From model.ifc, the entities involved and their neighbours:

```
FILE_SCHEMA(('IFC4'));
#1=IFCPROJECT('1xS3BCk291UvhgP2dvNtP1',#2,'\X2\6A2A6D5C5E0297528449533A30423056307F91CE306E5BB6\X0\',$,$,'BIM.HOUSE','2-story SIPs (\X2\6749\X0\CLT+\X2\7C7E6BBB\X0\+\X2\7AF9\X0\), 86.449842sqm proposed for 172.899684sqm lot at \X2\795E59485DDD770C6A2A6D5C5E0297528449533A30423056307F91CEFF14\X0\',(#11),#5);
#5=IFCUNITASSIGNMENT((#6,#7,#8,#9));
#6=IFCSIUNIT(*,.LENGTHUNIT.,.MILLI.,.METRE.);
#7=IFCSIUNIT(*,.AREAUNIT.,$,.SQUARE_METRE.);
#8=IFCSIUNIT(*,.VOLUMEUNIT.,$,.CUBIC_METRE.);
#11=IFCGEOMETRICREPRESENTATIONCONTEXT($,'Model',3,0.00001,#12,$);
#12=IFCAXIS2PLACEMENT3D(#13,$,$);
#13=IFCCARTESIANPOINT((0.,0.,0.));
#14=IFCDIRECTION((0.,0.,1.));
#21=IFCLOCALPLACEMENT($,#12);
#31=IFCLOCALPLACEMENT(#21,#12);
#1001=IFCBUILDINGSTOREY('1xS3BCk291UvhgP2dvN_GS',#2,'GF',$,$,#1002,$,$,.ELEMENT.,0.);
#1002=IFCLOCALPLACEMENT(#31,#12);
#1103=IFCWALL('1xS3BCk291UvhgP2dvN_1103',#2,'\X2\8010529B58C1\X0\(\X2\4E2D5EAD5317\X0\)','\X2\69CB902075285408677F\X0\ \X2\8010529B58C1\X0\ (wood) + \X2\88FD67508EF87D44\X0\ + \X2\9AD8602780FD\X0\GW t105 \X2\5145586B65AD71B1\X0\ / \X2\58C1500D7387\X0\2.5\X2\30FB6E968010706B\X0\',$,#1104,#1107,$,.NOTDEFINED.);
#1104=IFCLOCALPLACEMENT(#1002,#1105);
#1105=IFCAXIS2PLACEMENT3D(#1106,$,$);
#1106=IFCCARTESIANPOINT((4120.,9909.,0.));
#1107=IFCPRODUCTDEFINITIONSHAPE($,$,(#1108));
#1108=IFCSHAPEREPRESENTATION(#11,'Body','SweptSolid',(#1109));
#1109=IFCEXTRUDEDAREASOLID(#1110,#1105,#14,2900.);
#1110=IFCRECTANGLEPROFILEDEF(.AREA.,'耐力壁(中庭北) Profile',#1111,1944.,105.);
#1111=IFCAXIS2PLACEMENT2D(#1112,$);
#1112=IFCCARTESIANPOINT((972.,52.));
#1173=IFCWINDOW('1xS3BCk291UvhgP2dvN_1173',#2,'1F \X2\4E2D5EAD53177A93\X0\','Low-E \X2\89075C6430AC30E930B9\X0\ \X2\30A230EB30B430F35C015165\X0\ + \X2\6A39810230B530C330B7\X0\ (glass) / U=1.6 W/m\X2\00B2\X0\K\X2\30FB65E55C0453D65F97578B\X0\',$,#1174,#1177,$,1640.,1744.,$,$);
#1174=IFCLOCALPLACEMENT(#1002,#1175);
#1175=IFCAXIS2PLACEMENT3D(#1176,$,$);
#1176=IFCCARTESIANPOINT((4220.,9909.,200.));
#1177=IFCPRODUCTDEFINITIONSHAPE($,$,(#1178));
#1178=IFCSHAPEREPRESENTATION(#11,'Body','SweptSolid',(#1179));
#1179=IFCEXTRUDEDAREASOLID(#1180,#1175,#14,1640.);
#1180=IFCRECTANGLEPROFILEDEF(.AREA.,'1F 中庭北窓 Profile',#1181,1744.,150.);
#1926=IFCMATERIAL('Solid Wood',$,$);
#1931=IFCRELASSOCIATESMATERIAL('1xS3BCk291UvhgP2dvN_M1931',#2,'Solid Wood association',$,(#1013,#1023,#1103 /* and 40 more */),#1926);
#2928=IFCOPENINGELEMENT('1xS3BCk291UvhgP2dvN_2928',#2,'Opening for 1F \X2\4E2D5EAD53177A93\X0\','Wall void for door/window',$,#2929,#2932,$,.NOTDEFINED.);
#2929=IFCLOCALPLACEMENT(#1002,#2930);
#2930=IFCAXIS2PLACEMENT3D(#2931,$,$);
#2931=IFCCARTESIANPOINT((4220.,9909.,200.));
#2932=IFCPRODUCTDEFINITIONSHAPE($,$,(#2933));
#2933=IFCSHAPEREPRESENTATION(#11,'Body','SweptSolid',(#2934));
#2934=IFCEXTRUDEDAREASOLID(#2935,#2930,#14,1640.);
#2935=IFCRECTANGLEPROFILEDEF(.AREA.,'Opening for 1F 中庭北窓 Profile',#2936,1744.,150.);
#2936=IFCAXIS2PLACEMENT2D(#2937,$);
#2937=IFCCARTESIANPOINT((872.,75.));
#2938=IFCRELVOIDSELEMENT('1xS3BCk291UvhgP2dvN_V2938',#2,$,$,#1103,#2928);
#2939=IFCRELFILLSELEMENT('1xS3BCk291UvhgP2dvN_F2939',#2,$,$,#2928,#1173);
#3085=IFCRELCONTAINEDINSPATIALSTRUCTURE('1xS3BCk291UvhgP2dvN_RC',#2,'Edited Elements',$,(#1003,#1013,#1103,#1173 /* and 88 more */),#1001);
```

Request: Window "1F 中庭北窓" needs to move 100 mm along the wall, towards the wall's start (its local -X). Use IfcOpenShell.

```python
import ifcopenshell
import ifcopenshell.api.geometry
import ifcopenshell.util.placement
import ifcopenshell.util.unit

model = ifcopenshell.open("model.ifc")
unit_scale = ifcopenshell.util.unit.calculate_unit_scale(model)

window = model.by_guid("1xS3BCk291UvhgP2dvN_1173")
opening = window.FillsVoids[0].RelatingOpeningElement
wall = opening.VoidsElements[0].RelatingBuildingElement

wall_matrix = ifcopenshell.util.placement.get_local_placement(wall.ObjectPlacement)
shift = wall_matrix[:3, 0] * -0.1 / unit_scale
before = ifcopenshell.util.placement.get_local_placement(window.ObjectPlacement)[:3, 3].copy()

# The window is not placed relative to its opening, so move both.
for product in (opening, window):
    matrix = ifcopenshell.util.placement.get_local_placement(product.ObjectPlacement)
    matrix[:3, 3] += shift
    ifcopenshell.api.geometry.edit_object_placement(model, product=product, matrix=matrix, is_si=False)

after = ifcopenshell.util.placement.get_local_placement(window.ObjectPlacement)[:3, 3]
print("window moved by", (after - before).round(3) + 0.0)

model.write("model_v2.ifc")
```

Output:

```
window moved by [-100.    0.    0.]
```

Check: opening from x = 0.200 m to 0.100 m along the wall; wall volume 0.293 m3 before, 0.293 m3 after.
